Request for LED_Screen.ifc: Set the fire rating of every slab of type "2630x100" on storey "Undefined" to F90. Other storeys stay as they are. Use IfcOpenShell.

First a look at what the model holds.

```python
import ifcopenshell
import ifcopenshell.util.element

model = ifcopenshell.open("LED_Screen.ifc")
print(model.schema)
storey = next(s for s in model.by_type("IfcBuildingStorey") if s.Name == "Undefined")
slabs = [e for e in ifcopenshell.util.element.get_decomposition(storey) if e.is_a("IfcSlab")]
seen = {}
for e in slabs:
    element_type = ifcopenshell.util.element.get_type(e)
    key = (element_type.Name if element_type != e and element_type else None, ifcopenshell.util.element.get_pset(e, "Pset_SlabCommon", "FireRating"))
    seen[key] = seen.get(key, 0) + 1
for (name, value), count in sorted(seen.items(), key=str):
    print(count, "x", name, "|", value)
```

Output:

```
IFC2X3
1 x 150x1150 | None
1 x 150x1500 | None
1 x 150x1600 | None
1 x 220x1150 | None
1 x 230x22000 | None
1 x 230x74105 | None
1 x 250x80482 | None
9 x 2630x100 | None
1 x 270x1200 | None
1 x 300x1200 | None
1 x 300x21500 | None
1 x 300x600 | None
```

```python
import ifcopenshell
import ifcopenshell.api.pset
import ifcopenshell.util.element

model = ifcopenshell.open("LED_Screen.ifc")

storey = next(s for s in model.by_type("IfcBuildingStorey") if s.Name == "Undefined")
slabs = [e for e in ifcopenshell.util.element.get_decomposition(storey) if e.is_a("IfcSlab")]

count = 0
for e in slabs:
    element_type = ifcopenshell.util.element.get_type(e)
    if element_type in (None, e) or element_type.Name != "2630x100":
        continue
    found = ifcopenshell.util.element.get_pset(e, "Pset_SlabCommon", should_inherit=False)
    if found:
        pset = model.by_id(found["id"])
        if len(ifcopenshell.util.element.get_elements_by_pset(pset)) > 1:
            pset = ifcopenshell.api.pset.unshare_pset(model, products=[e], pset=pset)[0]
    else:
        pset = ifcopenshell.api.pset.add_pset(model, product=e, name="Pset_SlabCommon")
    ifcopenshell.api.pset.edit_pset(model, pset=pset, properties={"FireRating": "F90"})
    count += 1

print(count, "slabs updated")

model.write("LED_Screen_updated.ifc")
```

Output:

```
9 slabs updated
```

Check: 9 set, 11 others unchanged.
